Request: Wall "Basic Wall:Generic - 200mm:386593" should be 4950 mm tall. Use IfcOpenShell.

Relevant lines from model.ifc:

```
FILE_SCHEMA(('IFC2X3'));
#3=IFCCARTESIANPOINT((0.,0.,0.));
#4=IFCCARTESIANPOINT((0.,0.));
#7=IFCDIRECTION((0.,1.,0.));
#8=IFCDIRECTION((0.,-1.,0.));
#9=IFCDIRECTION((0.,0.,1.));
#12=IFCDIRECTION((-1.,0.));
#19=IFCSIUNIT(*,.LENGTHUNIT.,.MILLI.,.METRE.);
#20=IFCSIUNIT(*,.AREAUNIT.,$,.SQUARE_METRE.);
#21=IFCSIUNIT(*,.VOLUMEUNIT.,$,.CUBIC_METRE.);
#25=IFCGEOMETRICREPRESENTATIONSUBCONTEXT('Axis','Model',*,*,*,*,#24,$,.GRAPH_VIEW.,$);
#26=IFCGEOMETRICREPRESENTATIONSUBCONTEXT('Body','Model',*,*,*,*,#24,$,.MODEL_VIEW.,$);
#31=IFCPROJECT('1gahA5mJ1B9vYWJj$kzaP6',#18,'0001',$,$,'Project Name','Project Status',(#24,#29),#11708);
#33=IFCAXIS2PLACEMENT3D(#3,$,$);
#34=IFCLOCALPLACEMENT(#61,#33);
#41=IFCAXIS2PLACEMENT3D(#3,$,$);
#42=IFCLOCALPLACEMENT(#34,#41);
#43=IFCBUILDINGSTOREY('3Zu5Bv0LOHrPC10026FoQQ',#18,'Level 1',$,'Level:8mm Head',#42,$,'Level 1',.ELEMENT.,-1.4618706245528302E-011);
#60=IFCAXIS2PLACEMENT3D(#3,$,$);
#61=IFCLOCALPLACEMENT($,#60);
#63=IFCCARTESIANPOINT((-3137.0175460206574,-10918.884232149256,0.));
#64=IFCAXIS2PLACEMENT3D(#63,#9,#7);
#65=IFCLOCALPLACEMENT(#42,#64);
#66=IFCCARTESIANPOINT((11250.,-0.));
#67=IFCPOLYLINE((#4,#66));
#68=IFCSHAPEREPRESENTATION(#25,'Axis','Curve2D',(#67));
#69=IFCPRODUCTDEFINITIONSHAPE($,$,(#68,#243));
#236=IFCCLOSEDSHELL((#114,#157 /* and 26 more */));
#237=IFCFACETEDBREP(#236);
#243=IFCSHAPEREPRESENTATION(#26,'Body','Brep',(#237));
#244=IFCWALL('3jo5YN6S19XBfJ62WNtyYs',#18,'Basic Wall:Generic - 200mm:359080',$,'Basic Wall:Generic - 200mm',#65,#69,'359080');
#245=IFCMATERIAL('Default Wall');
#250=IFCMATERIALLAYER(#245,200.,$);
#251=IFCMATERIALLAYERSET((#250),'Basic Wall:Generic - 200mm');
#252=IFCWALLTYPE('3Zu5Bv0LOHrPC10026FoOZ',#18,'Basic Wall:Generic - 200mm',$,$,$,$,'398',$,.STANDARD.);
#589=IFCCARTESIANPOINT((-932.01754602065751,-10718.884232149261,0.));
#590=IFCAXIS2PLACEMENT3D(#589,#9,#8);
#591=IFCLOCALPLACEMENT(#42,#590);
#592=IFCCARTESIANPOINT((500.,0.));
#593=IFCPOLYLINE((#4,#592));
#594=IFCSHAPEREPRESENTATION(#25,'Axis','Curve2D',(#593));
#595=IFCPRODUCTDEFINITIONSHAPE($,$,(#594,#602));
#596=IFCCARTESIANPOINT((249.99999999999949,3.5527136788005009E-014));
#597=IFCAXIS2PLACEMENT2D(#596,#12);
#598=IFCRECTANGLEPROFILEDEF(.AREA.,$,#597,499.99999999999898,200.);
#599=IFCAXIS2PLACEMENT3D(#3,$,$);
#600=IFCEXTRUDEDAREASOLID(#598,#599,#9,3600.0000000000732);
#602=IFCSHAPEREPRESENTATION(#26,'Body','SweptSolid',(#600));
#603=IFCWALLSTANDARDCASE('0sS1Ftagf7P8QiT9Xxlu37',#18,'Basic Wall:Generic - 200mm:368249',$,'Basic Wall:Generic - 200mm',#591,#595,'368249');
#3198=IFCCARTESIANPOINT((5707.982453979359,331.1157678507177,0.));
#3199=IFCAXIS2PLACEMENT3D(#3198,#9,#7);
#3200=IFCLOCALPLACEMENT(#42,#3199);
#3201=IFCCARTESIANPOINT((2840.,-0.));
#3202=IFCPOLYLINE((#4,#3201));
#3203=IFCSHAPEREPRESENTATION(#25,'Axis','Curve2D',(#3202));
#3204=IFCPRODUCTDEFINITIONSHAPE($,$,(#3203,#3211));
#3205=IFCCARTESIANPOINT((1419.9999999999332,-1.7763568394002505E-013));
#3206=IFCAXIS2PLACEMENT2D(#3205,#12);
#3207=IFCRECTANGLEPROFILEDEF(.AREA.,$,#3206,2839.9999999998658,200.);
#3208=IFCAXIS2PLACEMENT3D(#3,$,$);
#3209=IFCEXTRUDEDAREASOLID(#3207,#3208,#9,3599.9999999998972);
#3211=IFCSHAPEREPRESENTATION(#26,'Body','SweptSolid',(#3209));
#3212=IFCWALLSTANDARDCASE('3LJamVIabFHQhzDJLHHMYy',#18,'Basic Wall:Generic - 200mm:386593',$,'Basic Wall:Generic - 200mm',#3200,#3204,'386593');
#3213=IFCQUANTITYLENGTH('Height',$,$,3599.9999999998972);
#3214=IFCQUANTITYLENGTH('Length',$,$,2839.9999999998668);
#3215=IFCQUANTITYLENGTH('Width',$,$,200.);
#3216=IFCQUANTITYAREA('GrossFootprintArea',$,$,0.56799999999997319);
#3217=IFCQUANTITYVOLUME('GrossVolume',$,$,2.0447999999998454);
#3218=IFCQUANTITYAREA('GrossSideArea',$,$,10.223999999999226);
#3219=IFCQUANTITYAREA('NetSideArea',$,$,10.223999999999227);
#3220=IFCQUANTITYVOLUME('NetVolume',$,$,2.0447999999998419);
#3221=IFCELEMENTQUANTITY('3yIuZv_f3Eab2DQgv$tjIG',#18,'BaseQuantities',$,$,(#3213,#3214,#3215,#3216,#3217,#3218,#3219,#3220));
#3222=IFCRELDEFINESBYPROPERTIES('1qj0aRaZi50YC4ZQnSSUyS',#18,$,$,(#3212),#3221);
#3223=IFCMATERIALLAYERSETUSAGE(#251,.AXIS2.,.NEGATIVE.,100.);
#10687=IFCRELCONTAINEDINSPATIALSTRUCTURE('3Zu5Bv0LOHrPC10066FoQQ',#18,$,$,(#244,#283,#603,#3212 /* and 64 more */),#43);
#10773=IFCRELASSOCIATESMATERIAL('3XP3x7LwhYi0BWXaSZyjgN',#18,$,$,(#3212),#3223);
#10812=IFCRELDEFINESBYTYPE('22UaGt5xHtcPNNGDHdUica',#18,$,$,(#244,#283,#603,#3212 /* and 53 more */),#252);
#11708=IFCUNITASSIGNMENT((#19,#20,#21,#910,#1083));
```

```python
import ifcopenshell
import ifcopenshell.api.pset
import ifcopenshell.geom
import ifcopenshell.util.element
import ifcopenshell.util.representation
import ifcopenshell.util.shape
import ifcopenshell.util.unit

model = ifcopenshell.open("model.ifc")
unit_scale = ifcopenshell.util.unit.calculate_unit_scale(model)
area_scale = ifcopenshell.util.unit.calculate_unit_scale(model, "AREAUNIT")
volume_scale = ifcopenshell.util.unit.calculate_unit_scale(model, "VOLUMEUNIT")
settings = ifcopenshell.geom.settings()


def volume(element):
    """Net volume in cubic metres, openings subtracted."""
    shape = ifcopenshell.geom.create_shape(settings, element)
    return ifcopenshell.util.shape.get_volume(shape.geometry)


wall = model.by_guid("3LJamVIabFHQhzDJLHHMYy")
before = volume(wall)

body = ifcopenshell.util.representation.get_representation(wall, "Model", "Body")
solid = body.Items[0]
old_height = solid.Depth
solid.Depth = 4950.0
after = volume(wall)
thickness = 0.2  # wall thickness in metres

# Update the stored height, areas and volumes.
qto = model.by_id(ifcopenshell.util.element.get_pset(wall, "BaseQuantities", should_inherit=False)["id"])
ifcopenshell.api.pset.edit_qto(model, qto=qto, properties={
    "Height": solid.Depth,
    "GrossVolume": ifcopenshell.util.element.get_pset(wall, "BaseQuantities", "GrossVolume") * solid.Depth / old_height,
    "GrossSideArea": ifcopenshell.util.element.get_pset(wall, "BaseQuantities", "GrossSideArea") * solid.Depth / old_height,
    "NetSideArea": after / thickness / area_scale,
    "NetVolume": after / volume_scale,
})

print(f"height {old_height:g} -> {solid.Depth:g}, volume {before:.3f} -> {after:.3f} m3")

model.write("model-out.ifc")
```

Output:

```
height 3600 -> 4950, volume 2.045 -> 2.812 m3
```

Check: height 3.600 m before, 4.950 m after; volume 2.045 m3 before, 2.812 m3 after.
